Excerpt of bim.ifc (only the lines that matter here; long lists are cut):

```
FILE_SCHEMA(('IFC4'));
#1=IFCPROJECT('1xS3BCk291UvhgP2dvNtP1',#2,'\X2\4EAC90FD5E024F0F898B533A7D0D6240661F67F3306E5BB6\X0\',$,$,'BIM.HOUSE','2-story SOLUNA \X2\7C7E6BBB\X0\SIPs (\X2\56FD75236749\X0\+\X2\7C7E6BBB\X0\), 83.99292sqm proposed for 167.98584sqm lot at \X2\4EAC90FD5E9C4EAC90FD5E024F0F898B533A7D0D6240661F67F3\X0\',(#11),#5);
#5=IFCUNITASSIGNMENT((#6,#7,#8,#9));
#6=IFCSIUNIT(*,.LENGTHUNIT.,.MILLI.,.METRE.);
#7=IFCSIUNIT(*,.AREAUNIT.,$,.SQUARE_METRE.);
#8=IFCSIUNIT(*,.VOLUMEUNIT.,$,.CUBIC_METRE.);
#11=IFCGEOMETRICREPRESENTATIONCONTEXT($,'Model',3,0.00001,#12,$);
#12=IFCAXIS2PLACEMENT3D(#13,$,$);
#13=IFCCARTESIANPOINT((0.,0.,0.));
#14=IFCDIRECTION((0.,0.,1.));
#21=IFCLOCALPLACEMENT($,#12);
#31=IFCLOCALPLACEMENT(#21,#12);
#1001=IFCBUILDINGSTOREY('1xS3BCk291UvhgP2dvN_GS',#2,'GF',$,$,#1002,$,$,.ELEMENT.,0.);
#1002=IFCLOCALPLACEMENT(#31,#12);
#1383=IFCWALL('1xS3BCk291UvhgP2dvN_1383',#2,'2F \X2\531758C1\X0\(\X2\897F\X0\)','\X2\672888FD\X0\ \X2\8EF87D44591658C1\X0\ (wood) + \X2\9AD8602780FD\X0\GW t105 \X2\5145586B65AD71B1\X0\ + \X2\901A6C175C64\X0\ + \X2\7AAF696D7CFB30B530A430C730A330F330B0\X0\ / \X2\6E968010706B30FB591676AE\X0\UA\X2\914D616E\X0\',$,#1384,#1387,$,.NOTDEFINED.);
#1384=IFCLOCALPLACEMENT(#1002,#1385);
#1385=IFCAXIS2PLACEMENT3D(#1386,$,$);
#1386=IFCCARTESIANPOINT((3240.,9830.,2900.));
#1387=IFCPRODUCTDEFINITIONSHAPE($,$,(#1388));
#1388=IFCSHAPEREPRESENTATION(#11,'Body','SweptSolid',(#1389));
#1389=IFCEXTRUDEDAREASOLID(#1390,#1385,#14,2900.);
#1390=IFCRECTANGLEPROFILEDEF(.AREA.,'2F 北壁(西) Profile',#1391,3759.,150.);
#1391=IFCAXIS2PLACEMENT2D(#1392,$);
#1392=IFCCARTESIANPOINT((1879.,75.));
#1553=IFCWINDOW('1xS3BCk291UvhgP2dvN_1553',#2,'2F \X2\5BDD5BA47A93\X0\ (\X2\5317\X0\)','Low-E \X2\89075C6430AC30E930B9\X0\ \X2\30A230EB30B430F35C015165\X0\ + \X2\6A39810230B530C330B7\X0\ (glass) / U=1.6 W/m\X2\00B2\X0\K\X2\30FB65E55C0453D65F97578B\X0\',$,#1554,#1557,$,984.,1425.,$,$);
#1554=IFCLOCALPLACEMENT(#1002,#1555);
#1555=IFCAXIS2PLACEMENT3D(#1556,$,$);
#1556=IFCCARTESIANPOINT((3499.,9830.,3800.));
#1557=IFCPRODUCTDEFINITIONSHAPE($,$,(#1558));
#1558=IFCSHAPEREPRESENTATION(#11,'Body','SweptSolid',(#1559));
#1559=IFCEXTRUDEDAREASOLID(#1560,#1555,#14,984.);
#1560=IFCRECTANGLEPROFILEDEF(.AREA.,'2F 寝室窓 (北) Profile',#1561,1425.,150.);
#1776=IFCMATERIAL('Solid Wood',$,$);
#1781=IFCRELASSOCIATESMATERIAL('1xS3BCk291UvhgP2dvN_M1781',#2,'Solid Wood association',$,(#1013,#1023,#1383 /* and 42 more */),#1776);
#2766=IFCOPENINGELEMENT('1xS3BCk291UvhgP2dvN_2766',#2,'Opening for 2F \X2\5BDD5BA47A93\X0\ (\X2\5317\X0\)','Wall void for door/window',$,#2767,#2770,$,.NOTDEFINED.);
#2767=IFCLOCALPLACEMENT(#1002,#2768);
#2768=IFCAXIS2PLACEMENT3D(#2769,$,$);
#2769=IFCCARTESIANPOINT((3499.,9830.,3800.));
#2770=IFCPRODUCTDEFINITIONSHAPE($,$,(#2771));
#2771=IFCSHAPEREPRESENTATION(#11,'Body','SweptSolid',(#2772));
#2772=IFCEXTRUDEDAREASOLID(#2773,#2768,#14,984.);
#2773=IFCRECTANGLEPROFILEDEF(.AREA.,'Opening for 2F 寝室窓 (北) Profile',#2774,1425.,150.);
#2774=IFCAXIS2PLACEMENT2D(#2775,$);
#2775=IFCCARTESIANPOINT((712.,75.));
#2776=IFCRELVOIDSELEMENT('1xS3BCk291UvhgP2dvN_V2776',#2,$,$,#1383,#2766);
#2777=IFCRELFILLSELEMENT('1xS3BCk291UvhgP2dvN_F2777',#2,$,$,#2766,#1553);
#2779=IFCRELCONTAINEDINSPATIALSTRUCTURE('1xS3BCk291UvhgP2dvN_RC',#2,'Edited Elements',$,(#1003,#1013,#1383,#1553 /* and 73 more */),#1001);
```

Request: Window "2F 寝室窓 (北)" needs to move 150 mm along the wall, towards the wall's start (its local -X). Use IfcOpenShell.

```python
import ifcopenshell
import ifcopenshell.api.geometry
import ifcopenshell.util.placement
import ifcopenshell.util.unit

model = ifcopenshell.open("bim.ifc")
unit_scale = ifcopenshell.util.unit.calculate_unit_scale(model)

window = model.by_id(1553)
opening = window.FillsVoids[0].RelatingOpeningElement
wall = opening.VoidsElements[0].RelatingBuildingElement

wall_matrix = ifcopenshell.util.placement.get_local_placement(wall.ObjectPlacement)
shift = wall_matrix[:3, 0] * -0.15 / unit_scale
before = ifcopenshell.util.placement.get_local_placement(window.ObjectPlacement)[:3, 3].copy()

# The window is not placed relative to its opening, so move both.
for product in (opening, window):
    matrix = ifcopenshell.util.placement.get_local_placement(product.ObjectPlacement)
    matrix[:3, 3] += shift
    ifcopenshell.api.geometry.edit_object_placement(model, product=product, matrix=matrix, is_si=False)

after = ifcopenshell.util.placement.get_local_placement(window.ObjectPlacement)[:3, 3]
print("window moved by", (after - before).round(3) + 0.0)

model.write("bim_updated.ifc")
```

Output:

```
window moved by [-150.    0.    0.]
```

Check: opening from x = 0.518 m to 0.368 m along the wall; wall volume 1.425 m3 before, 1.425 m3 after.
